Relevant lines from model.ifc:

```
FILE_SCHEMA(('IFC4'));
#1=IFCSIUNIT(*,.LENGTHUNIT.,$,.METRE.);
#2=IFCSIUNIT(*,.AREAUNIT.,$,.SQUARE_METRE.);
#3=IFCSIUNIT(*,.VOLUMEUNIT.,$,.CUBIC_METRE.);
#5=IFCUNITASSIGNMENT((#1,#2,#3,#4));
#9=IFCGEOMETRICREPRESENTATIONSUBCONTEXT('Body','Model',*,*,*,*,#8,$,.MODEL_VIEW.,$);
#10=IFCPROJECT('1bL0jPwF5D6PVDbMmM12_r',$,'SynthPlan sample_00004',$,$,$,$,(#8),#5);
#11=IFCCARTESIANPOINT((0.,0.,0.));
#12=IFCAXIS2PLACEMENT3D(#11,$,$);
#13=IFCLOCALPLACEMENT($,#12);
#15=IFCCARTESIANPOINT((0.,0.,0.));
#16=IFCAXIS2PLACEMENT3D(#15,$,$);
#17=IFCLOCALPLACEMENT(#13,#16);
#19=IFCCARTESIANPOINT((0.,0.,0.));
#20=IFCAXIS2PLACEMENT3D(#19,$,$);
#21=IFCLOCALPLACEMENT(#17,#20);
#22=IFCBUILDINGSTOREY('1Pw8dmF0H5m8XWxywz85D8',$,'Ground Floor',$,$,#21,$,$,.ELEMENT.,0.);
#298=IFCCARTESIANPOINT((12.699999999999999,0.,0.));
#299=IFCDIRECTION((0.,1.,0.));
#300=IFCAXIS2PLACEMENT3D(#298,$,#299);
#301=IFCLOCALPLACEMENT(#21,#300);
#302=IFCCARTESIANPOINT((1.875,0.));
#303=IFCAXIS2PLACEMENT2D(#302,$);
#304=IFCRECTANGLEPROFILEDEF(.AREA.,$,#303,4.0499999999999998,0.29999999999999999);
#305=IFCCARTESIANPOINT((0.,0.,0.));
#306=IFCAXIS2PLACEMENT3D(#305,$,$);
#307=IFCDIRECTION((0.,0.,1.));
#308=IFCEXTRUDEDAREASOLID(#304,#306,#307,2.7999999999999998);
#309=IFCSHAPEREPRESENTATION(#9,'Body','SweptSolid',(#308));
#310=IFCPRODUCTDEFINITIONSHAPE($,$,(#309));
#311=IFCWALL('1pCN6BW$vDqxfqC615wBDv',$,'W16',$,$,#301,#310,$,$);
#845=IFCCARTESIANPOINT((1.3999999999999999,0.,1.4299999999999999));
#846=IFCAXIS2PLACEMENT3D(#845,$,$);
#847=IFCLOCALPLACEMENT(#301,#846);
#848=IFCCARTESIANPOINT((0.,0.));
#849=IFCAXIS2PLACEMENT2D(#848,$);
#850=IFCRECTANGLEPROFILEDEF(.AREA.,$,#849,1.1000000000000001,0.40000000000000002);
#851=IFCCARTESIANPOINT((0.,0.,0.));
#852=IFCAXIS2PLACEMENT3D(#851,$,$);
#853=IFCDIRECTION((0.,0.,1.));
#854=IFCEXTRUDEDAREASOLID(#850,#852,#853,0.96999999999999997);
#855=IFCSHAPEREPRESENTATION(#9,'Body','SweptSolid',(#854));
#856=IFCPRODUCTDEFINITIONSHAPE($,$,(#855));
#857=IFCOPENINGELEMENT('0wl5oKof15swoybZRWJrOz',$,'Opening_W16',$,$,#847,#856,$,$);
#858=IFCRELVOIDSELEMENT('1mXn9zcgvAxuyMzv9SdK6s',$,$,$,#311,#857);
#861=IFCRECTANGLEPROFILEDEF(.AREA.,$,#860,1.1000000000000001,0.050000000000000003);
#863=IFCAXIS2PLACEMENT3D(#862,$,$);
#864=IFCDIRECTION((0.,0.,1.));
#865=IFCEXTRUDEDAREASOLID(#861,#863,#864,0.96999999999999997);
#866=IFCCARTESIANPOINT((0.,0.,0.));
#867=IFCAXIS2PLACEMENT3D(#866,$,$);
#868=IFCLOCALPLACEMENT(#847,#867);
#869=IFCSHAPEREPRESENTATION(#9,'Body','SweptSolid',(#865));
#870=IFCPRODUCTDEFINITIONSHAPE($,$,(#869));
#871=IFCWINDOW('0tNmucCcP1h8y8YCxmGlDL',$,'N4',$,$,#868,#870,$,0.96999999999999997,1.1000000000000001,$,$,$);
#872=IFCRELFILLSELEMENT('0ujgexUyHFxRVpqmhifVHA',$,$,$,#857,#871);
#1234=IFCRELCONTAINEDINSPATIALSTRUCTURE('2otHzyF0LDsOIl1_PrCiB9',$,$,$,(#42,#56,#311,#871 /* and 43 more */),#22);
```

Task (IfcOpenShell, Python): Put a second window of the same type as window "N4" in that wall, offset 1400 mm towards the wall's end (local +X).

```python
import ifcopenshell
import ifcopenshell.api.feature
import ifcopenshell.api.geometry
import ifcopenshell.api.root
import ifcopenshell.geom
import ifcopenshell.util.element
import ifcopenshell.util.placement
import ifcopenshell.util.shape
import ifcopenshell.util.unit

model = ifcopenshell.open("model.ifc")
unit_scale = ifcopenshell.util.unit.calculate_unit_scale(model)
settings = ifcopenshell.geom.settings()


def volume(element):
    """Net volume in cubic metres, openings subtracted."""
    shape = ifcopenshell.geom.create_shape(settings, element)
    return ifcopenshell.util.shape.get_volume(shape.geometry)


window = model.by_guid("0tNmucCcP1h8y8YCxmGlDL")
opening = window.FillsVoids[0].RelatingOpeningElement
wall = opening.VoidsElements[0].RelatingBuildingElement
before = volume(wall)
shift = ifcopenshell.util.placement.get_local_placement(wall.ObjectPlacement)[:3, 0] * 1.4 / unit_scale

# copy_class copies the void relationship, type, container and properties, but no geometry.
new_opening = ifcopenshell.api.root.copy_class(model, product=opening)
new_opening.Representation = ifcopenshell.util.element.copy_deep(
    model, opening.Representation, exclude=["IfcGeometricRepresentationContext", "IfcRepresentationMap"]
)
new_window = ifcopenshell.api.root.copy_class(model, product=window)
new_window.Representation = ifcopenshell.util.element.copy_deep(
    model, window.Representation, exclude=["IfcGeometricRepresentationContext", "IfcRepresentationMap"]
)
ifcopenshell.api.feature.add_filling(model, opening=new_opening, element=new_window)

for old, new in ((opening, new_opening), (window, new_window)):
    matrix = ifcopenshell.util.placement.get_local_placement(old.ObjectPlacement)
    matrix[:3, 3] += shift
    ifcopenshell.api.geometry.edit_object_placement(model, product=new, matrix=matrix, is_si=False)

after = volume(wall)

print(f"wall volume {before:.3f} -> {after:.3f} m3")

model.write("model_updated.ifc")
```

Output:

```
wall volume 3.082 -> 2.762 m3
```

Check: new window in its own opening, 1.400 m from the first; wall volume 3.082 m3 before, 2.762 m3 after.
